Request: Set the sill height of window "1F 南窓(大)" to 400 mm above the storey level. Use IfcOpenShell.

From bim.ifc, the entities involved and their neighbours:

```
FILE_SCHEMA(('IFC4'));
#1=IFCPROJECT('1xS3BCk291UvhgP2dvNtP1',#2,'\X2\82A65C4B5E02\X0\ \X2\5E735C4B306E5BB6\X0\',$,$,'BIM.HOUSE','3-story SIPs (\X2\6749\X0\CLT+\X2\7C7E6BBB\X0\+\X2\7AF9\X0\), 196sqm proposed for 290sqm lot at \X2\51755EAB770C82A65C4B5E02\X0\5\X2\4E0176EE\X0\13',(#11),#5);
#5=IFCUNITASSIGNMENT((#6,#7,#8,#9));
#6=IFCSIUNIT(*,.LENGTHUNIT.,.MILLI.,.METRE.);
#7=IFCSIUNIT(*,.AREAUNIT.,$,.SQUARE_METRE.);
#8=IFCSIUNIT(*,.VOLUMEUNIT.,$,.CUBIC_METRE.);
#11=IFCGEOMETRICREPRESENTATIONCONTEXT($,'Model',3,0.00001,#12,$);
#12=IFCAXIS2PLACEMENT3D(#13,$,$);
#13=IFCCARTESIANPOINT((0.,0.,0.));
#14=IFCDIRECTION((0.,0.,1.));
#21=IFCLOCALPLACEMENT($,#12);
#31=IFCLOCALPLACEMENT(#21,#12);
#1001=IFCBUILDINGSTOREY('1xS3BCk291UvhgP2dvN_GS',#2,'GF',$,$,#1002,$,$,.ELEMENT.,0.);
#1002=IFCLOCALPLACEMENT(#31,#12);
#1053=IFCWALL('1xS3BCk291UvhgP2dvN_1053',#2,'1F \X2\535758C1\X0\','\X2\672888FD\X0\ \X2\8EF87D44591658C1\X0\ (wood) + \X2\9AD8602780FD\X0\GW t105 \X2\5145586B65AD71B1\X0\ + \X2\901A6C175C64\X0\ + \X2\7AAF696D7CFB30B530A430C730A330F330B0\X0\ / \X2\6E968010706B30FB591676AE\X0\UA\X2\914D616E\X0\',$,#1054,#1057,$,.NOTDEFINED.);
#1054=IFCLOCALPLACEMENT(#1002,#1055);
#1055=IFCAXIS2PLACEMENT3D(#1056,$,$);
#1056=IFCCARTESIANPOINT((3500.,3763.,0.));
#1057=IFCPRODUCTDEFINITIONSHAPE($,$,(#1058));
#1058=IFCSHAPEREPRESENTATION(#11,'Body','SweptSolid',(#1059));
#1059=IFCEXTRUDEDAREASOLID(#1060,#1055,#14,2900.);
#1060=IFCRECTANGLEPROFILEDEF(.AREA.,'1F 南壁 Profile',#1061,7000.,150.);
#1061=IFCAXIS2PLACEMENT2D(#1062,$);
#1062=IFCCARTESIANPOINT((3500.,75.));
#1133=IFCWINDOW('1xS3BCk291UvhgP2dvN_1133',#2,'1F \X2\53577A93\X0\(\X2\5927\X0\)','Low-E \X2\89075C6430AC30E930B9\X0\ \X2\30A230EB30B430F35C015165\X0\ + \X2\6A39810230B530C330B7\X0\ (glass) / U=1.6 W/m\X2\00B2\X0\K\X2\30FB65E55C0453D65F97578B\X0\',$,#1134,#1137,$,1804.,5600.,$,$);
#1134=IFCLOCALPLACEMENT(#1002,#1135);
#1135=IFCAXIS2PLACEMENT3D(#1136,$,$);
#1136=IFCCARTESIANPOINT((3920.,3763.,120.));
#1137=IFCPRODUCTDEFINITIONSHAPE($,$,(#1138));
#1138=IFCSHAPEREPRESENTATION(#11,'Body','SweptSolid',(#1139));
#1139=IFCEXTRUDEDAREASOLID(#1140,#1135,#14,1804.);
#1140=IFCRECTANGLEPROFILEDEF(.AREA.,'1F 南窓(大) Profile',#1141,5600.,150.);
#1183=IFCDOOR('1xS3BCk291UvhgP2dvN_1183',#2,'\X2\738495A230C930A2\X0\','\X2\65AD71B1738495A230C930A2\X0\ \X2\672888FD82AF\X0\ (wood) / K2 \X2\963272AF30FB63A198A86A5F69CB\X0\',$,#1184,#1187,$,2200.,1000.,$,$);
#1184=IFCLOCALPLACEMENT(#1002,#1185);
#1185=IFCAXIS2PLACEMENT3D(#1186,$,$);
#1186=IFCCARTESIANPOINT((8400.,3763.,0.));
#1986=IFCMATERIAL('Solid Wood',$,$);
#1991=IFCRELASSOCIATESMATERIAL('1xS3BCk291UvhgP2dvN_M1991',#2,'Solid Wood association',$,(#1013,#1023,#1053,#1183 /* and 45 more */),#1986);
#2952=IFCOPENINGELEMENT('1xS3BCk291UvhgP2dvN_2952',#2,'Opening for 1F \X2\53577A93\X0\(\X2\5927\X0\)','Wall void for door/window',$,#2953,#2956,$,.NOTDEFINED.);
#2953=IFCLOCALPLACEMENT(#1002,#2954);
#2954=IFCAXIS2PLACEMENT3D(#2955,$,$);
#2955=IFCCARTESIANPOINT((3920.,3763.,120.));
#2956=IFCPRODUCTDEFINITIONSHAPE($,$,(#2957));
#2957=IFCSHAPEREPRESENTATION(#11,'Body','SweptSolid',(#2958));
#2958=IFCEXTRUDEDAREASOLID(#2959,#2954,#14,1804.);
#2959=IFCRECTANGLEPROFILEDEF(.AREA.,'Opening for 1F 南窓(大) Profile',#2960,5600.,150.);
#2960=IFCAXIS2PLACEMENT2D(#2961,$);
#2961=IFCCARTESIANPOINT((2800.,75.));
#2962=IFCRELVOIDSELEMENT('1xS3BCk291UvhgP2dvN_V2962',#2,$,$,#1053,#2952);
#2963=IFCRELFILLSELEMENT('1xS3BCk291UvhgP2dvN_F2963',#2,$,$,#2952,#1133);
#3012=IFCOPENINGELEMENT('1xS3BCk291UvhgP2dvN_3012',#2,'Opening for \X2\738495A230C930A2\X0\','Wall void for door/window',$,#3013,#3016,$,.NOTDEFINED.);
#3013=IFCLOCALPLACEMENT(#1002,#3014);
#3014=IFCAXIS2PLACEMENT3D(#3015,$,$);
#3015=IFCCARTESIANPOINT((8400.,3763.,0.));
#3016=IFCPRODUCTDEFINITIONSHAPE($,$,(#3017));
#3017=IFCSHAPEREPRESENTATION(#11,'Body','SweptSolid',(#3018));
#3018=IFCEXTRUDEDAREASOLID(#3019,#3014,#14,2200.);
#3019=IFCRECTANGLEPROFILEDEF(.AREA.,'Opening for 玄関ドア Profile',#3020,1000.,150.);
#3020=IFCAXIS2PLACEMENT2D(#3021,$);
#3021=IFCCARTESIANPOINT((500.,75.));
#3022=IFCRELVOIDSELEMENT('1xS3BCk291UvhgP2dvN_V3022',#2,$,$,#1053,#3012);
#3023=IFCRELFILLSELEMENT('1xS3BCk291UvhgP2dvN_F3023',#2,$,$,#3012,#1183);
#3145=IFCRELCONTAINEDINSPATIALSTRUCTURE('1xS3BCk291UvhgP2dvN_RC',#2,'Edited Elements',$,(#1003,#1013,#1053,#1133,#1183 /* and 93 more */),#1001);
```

```python
import numpy as np
import ifcopenshell
import ifcopenshell.api.geometry
import ifcopenshell.geom
import ifcopenshell.util.element
import ifcopenshell.util.placement
import ifcopenshell.util.shape
import ifcopenshell.util.unit

model = ifcopenshell.open("bim.ifc")
unit_scale = ifcopenshell.util.unit.calculate_unit_scale(model)

window = model.by_guid("1xS3BCk291UvhgP2dvN_1133")
opening = window.FillsVoids[0].RelatingOpeningElement
storey = ifcopenshell.util.element.get_container(window, ifc_class="IfcBuildingStorey")
level = ifcopenshell.util.placement.get_local_placement(storey.ObjectPlacement)[2, 3]

# The opening's origin need not be at the sill, so measure its lowest point.
shape = ifcopenshell.geom.create_shape(ifcopenshell.geom.settings(), opening)
bottom = ifcopenshell.util.shape.get_shape_bottom_elevation(shape, shape.geometry) / unit_scale
dz = level + 400.0 - bottom

shift = np.array([0.0, 0.0, dz])
# The window is not placed relative to its opening, so move both.
for product in (opening, window):
    matrix = ifcopenshell.util.placement.get_local_placement(product.ObjectPlacement)
    matrix[:3, 3] += shift
    ifcopenshell.api.geometry.edit_object_placement(model, product=product, matrix=matrix, is_si=False)

print(f"moved by {dz * unit_scale:+.3f} m")

model.write("bim_edited.ifc")
```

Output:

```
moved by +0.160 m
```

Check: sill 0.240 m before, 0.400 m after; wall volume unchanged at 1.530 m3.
